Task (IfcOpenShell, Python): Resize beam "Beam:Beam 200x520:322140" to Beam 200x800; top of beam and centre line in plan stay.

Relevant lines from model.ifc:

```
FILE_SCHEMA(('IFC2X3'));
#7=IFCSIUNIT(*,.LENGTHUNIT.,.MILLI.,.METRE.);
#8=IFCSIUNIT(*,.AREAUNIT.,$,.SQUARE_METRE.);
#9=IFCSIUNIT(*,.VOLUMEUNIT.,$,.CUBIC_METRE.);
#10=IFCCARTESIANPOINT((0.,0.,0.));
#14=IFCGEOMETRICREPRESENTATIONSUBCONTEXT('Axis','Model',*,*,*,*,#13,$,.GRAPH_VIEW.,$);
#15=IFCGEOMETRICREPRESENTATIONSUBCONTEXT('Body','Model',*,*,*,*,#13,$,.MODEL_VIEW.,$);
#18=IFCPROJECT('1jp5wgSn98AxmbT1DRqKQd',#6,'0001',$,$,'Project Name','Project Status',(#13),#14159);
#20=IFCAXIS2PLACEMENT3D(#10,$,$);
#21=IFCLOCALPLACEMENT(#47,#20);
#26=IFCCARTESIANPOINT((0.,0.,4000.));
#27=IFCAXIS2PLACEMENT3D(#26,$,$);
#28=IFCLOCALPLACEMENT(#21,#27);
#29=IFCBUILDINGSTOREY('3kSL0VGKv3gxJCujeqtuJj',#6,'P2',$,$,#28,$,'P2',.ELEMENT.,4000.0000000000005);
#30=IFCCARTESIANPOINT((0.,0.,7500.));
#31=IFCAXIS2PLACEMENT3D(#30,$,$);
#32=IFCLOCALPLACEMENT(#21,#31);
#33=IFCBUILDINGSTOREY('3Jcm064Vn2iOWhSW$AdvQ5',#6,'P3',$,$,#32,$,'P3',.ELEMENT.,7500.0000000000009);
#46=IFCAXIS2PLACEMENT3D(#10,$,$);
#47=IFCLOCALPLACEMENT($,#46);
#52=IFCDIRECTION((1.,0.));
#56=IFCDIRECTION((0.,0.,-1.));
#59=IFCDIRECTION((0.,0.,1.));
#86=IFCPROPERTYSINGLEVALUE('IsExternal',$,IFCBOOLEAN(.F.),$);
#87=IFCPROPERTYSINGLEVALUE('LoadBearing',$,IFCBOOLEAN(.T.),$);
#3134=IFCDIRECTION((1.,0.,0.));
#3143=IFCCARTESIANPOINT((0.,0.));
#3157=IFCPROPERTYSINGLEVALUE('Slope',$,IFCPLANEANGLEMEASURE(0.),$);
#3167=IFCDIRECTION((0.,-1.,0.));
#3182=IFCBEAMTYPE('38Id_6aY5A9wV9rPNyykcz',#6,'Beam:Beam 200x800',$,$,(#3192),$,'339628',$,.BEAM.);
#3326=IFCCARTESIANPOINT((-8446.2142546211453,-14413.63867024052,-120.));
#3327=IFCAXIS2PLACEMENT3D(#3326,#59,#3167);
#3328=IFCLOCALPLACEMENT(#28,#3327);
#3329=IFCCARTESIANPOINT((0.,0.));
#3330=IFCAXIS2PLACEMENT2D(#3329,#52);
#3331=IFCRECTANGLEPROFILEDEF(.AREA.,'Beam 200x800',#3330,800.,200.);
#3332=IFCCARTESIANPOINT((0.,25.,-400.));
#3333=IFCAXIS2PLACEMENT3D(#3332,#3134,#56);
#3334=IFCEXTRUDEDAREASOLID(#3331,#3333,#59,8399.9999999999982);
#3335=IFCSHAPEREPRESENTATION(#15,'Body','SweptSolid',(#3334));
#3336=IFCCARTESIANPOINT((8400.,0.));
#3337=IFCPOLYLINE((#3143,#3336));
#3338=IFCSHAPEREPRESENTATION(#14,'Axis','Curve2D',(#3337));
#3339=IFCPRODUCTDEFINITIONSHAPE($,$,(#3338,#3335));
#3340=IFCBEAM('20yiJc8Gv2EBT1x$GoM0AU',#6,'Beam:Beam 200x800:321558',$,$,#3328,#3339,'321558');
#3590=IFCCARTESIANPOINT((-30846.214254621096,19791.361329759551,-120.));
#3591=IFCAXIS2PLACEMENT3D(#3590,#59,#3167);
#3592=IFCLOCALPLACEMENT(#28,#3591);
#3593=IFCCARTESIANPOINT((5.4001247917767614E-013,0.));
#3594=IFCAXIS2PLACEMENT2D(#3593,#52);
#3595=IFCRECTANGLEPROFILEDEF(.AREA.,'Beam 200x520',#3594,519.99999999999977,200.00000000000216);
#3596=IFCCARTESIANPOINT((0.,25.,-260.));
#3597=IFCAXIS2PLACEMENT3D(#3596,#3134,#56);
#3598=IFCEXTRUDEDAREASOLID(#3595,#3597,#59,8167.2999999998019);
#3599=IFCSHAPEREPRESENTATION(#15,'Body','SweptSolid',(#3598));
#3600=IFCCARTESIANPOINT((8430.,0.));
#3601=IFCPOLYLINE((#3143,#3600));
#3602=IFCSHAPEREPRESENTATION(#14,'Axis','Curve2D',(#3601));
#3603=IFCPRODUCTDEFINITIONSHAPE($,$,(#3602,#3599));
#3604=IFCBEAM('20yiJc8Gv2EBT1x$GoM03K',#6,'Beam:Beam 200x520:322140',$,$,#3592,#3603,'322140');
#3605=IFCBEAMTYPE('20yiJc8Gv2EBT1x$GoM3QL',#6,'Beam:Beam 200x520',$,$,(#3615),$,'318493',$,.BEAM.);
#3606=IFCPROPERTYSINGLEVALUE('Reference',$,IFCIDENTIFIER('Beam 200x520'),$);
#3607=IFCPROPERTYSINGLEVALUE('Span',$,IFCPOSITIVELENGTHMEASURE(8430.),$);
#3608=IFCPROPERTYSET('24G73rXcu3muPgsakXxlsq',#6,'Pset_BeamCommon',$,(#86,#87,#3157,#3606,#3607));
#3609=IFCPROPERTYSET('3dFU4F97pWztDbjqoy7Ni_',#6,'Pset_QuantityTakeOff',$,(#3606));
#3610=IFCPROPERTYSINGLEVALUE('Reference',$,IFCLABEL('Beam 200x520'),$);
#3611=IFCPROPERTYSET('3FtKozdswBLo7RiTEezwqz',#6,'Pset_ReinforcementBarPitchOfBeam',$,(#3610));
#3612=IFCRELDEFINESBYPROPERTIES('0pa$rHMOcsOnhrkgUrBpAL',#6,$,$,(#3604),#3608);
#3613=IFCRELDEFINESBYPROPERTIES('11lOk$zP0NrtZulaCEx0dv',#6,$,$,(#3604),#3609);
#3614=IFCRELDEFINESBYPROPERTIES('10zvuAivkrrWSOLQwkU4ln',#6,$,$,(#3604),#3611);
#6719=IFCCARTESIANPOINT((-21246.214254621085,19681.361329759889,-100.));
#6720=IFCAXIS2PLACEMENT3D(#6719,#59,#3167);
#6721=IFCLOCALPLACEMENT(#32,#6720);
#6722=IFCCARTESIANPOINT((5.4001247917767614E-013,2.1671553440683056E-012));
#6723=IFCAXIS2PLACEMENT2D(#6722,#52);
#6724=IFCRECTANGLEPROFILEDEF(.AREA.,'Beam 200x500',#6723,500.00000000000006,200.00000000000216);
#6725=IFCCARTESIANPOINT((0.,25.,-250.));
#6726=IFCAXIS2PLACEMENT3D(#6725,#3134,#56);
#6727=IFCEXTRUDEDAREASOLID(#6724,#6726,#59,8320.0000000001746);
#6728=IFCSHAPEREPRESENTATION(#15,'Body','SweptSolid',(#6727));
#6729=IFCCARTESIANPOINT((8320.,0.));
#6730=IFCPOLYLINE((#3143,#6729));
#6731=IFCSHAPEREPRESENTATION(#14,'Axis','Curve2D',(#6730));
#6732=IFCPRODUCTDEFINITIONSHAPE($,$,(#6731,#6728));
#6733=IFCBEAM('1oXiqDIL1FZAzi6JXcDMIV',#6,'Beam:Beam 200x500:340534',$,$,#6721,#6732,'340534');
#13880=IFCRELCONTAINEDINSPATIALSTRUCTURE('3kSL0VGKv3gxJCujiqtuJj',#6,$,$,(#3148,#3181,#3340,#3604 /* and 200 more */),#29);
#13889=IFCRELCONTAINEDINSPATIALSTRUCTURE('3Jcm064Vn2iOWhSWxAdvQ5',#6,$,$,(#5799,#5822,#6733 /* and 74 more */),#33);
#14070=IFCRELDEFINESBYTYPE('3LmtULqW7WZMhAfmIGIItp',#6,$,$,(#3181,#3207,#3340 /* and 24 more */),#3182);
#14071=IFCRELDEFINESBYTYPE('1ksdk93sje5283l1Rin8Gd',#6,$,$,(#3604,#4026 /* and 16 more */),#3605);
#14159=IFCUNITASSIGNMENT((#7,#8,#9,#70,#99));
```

```python
import ifcopenshell
import ifcopenshell.api.pset
import ifcopenshell.api.type
import ifcopenshell.util.element
import ifcopenshell.util.representation

model = ifcopenshell.open("model.ifc")

member = model.by_guid("20yiJc8Gv2EBT1x$GoM03K")
source = next(p for p in model.by_type("IfcRectangleProfileDef") if p.ProfileName == "Beam 200x800")

body = ifcopenshell.util.representation.get_representation(member, "Model", "Body")
solid = body.Items[0]
old_profile = solid.SweptArea

# Copy the section's sizes but keep this member's own profile position.
profile = ifcopenshell.util.element.copy(model, source)
# Profiles are centred, so shift by half the change in depth to hold the top.
shift = (old_profile.XDim - profile.XDim) / 2
x, y = old_profile.Position.Location.Coordinates
up = (-1.0, 0.0)  # upwards, in the solid's own plane
location = model.createIfcCartesianPoint((x + up[0] * shift, y + up[1] * shift))
profile.Position = model.createIfcAxis2Placement2D(location, old_profile.Position.RefDirection)
solid.SweptArea = profile
if not model.get_total_inverses(old_profile):
    ifcopenshell.util.element.remove_deep2(model, old_profile)

new_type = model.by_guid("38Id_6aY5A9wV9rPNyykcz")
ifcopenshell.api.type.assign_type(
    model, related_objects=[member], relating_type=new_type, should_map_representations=False
)
member.Name = member.Name.replace("Beam 200x520", "Beam 200x800")
pset = model.by_id(ifcopenshell.util.element.get_pset(member, "Pset_BeamCommon", should_inherit=False)["id"])
ifcopenshell.api.pset.edit_pset(model, pset=pset, properties={"Reference": "Beam 200x800"})
pset = model.by_id(ifcopenshell.util.element.get_pset(member, "Pset_QuantityTakeOff", should_inherit=False)["id"])
ifcopenshell.api.pset.edit_pset(model, pset=pset, properties={"Reference": "Beam 200x800"})
pset = model.by_id(ifcopenshell.util.element.get_pset(member, "Pset_ReinforcementBarPitchOfBeam", should_inherit=False)["id"])
ifcopenshell.api.pset.edit_pset(model, pset=pset, properties={"Reference": "Beam 200x800"})

print(solid.SweptArea)

model.write("model-out.ifc")
```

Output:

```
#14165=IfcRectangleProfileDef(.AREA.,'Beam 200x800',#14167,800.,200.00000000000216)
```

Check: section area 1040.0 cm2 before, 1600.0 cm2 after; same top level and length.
